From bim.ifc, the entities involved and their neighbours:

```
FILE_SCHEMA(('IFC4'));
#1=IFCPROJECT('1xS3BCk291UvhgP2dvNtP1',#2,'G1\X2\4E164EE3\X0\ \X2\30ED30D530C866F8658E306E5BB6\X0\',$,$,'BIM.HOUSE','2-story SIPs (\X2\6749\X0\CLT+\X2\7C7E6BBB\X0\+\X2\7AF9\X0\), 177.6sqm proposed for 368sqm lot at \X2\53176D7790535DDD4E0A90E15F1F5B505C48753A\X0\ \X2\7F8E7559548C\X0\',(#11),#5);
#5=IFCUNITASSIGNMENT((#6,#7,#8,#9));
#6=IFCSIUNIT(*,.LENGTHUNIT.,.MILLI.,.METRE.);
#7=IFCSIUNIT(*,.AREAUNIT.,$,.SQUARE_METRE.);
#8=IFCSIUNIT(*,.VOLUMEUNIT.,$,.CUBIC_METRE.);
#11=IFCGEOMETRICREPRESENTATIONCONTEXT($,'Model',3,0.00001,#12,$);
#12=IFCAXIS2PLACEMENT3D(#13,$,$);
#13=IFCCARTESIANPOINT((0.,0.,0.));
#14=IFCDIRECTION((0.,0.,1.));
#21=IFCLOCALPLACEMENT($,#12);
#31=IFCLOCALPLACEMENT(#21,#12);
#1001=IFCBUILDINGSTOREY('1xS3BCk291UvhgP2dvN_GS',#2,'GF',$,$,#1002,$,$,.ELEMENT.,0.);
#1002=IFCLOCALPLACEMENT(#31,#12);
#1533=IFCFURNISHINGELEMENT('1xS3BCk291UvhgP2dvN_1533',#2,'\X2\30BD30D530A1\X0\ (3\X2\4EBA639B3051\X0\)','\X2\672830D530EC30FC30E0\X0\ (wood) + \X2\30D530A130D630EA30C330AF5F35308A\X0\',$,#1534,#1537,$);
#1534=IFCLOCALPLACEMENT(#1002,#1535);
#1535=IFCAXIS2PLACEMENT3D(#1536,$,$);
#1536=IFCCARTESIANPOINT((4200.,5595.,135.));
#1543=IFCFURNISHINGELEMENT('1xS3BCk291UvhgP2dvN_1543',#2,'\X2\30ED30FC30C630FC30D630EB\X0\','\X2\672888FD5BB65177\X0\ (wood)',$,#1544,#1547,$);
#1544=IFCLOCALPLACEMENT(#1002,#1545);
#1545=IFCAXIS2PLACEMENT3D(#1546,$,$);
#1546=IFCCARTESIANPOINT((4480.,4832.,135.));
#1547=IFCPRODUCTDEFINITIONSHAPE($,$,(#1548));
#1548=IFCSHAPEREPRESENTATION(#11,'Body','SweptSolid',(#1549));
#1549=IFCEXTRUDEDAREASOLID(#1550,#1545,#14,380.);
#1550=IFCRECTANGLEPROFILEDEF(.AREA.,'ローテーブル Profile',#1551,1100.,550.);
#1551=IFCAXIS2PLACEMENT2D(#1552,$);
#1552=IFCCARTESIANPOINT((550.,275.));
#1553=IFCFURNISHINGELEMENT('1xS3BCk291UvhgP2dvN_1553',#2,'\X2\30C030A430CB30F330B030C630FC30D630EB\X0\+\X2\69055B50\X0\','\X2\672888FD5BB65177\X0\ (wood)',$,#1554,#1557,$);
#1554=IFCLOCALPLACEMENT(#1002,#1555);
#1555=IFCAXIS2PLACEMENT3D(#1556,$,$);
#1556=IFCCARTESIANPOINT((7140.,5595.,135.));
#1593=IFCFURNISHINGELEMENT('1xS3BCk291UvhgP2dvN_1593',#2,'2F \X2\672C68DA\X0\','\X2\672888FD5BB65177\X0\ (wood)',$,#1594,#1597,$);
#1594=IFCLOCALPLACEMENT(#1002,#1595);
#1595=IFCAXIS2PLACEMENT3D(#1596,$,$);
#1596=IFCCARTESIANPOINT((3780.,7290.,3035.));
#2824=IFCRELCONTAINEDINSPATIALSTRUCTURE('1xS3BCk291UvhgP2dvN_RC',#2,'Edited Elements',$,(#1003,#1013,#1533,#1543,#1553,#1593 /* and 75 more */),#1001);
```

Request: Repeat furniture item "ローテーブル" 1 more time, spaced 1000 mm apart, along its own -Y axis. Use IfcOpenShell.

```python
import ifcopenshell
import ifcopenshell.api.geometry
import ifcopenshell.api.root
import ifcopenshell.util.element
import ifcopenshell.util.placement

model = ifcopenshell.open("bim.ifc")


def reuse_history(source, copy):
    """copy_class also copies each property set's owner history, people and application; keep the originals."""
    for rel in copy.IsDefinedBy:
        if rel.is_a("IfcRelDefinesByProperties") and (history := rel.RelatingPropertyDefinition.OwnerHistory):
            rel.RelatingPropertyDefinition.OwnerHistory = source.OwnerHistory
            ifcopenshell.util.element.remove_deep2(model, history)


source = model.by_guid("1xS3BCk291UvhgP2dvN_1543")
base = ifcopenshell.util.placement.get_local_placement(source.ObjectPlacement)
step = -base[:3, 1] * 1000.0

for i in range(1, 2):
    copy = ifcopenshell.api.root.copy_class(model, product=source)
    copy.Representation = ifcopenshell.util.element.copy_deep(
        model, source.Representation, exclude=["IfcGeometricRepresentationContext", "IfcRepresentationMap"]
    )
    reuse_history(source, copy)
    matrix = base.copy()
    matrix[:3, 3] += i * step
    print("added at", matrix[:3, 3].round(3) + 0.0)
    ifcopenshell.api.geometry.edit_object_placement(model, product=copy, matrix=matrix, is_si=False)

model.write("bim_rev.ifc")
```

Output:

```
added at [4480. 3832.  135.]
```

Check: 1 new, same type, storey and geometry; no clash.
